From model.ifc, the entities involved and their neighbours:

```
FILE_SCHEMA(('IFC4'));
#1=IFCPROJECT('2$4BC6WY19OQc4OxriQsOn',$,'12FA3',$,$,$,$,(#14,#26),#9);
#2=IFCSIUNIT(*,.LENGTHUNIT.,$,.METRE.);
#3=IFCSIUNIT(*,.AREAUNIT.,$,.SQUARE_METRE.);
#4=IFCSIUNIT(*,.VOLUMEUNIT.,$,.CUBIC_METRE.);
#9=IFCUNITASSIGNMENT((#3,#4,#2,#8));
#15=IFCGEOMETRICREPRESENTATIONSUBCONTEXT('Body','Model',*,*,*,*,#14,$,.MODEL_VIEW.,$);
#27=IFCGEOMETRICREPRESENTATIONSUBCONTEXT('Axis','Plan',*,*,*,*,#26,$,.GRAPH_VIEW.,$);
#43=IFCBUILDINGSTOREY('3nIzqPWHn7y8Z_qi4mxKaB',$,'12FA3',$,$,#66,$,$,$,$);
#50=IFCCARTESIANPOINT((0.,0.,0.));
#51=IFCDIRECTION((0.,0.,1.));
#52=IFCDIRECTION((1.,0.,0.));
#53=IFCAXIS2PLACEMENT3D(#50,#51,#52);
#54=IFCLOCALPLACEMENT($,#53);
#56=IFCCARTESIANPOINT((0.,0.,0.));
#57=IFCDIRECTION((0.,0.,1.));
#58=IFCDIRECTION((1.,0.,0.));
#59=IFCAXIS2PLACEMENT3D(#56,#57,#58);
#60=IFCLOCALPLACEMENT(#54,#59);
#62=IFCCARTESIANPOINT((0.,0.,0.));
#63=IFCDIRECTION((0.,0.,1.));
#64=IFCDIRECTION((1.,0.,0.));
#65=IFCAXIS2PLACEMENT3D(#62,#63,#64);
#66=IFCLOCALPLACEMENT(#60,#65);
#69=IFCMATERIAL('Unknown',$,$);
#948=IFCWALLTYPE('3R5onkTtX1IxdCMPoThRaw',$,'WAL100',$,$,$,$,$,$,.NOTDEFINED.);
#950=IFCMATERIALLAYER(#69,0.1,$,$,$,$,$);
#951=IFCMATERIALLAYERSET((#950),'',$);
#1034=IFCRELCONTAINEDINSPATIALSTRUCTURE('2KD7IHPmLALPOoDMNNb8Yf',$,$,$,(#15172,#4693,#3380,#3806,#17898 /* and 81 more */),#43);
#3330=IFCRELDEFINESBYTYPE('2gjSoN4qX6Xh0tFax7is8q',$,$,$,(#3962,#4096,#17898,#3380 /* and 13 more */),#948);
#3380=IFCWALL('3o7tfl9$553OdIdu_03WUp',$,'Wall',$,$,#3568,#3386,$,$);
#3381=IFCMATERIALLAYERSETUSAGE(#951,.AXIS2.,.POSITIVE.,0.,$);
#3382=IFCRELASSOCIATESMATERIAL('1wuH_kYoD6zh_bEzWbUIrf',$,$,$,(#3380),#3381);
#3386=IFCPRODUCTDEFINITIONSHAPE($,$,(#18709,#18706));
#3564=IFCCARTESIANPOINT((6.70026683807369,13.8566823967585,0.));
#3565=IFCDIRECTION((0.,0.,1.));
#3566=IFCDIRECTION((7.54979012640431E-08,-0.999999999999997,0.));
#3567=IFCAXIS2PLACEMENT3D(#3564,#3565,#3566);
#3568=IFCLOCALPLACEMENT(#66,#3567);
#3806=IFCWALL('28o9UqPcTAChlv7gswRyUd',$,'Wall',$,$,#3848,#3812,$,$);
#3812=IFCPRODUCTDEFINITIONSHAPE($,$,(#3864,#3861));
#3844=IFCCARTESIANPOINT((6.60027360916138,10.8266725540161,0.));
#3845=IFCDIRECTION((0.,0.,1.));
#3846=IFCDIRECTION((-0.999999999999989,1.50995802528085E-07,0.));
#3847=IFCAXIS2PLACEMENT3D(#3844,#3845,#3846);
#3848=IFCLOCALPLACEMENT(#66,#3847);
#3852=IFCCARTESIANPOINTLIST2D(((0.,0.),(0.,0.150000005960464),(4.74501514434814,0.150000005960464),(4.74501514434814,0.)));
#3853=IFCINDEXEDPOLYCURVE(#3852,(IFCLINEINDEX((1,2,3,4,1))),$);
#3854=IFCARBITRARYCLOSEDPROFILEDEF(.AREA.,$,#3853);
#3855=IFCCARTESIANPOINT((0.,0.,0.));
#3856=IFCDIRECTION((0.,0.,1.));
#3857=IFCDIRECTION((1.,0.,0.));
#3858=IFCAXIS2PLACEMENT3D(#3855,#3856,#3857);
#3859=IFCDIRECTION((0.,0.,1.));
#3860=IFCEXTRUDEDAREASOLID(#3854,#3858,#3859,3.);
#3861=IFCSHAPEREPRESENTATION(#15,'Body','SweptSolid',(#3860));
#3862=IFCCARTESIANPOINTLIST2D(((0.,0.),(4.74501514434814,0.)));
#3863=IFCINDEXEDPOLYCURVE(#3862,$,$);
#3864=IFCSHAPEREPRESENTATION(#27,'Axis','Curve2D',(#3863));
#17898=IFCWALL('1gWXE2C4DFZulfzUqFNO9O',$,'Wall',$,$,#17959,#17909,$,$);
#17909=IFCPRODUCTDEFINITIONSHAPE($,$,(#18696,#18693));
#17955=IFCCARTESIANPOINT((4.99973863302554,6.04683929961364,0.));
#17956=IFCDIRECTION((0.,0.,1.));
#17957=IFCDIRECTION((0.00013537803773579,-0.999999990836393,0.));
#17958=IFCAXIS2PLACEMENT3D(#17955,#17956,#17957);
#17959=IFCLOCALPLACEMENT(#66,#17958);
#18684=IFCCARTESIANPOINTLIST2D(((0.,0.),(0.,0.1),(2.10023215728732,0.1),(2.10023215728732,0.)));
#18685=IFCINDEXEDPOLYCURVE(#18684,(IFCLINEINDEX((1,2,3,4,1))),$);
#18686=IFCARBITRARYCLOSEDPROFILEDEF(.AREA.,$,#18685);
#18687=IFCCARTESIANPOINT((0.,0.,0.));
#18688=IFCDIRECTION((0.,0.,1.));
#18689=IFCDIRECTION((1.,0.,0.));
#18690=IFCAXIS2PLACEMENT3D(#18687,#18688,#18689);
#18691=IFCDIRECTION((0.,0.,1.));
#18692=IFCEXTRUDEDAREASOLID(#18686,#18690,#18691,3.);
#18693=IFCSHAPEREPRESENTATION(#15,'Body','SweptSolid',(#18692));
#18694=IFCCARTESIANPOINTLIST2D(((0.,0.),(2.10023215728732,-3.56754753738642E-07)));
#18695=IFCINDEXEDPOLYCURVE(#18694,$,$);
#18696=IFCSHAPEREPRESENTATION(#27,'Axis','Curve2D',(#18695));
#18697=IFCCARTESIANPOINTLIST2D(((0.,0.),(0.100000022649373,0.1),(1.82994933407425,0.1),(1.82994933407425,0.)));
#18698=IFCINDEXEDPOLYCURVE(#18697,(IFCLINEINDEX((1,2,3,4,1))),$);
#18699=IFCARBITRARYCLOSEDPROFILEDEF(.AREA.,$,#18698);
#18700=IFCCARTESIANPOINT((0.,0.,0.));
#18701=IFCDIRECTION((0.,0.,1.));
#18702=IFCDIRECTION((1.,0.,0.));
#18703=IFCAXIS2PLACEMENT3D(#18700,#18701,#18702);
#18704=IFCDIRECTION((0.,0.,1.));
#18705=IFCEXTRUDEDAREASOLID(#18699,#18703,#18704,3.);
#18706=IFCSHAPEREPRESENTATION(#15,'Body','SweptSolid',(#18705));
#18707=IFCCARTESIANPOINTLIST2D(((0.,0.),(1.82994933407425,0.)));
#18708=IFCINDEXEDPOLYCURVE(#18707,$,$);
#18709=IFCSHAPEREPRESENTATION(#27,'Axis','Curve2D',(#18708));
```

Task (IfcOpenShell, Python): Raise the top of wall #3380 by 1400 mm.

```python
import ifcopenshell
import ifcopenshell.geom
import ifcopenshell.util.representation
import ifcopenshell.util.shape
import ifcopenshell.util.unit

model = ifcopenshell.open("model.ifc")
unit_scale = ifcopenshell.util.unit.calculate_unit_scale(model)
settings = ifcopenshell.geom.settings()


def volume(element):
    """Net volume in cubic metres, openings subtracted."""
    shape = ifcopenshell.geom.create_shape(settings, element)
    return ifcopenshell.util.shape.get_volume(shape.geometry)


wall = model.by_guid("3o7tfl9$553OdIdu_03WUp")
before = volume(wall)

body = ifcopenshell.util.representation.get_representation(wall, "Model", "Body")
solid = body.Items[0]
old_height = solid.Depth
solid.Depth += 1.4 / unit_scale
after = volume(wall)

print(f"height {old_height:g} -> {solid.Depth:g}, volume {before:.3f} -> {after:.3f} m3")

model.write("model_edited.ifc")
```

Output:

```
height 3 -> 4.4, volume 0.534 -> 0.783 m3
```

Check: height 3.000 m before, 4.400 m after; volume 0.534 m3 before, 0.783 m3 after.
